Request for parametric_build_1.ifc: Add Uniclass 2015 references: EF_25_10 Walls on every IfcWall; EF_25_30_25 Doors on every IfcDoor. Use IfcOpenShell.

First a look at what the model holds.

```python
import ifcopenshell

model = ifcopenshell.open("parametric_build_1.ifc")
print(model.schema)
print("classifications:", [c.Name for c in model.by_type("IfcClassification")])
for ifc_class in ("IfcDoor", "IfcRoof", "IfcStair", "IfcWall", "IfcWindow"):
    print(ifc_class, len(model.by_type(ifc_class)))
```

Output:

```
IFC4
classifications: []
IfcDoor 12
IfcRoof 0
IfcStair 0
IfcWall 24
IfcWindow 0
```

```python
import ifcopenshell
import ifcopenshell.api.classification

model = ifcopenshell.open("parametric_build_1.ifc")

system = ifcopenshell.api.classification.add_classification(model, classification="Uniclass 2015")

codes = {
    "IfcWall": ("EF_25_10", "Walls"),
    "IfcDoor": ("EF_25_30_25", "Doors"),
}
for ifc_class, (code, name) in codes.items():
    products = model.by_type(ifc_class)
    ifcopenshell.api.classification.add_reference(
        model, products=products, classification=system, identification=code, name=name
    )
    print(code, len(products))

model.write("parametric_build_1_edited.ifc")
```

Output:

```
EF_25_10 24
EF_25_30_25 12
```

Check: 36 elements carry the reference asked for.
